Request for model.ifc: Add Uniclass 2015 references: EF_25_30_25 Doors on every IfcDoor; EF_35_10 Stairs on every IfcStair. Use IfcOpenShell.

First a look at what the model holds.

```python
import ifcopenshell

model = ifcopenshell.open("model.ifc")
print(model.schema)
print("classifications:", [c.Name for c in model.by_type("IfcClassification")])
for ifc_class in ("IfcDoor", "IfcRoof", "IfcStair", "IfcWall", "IfcWindow"):
    print(ifc_class, len(model.by_type(ifc_class)))
```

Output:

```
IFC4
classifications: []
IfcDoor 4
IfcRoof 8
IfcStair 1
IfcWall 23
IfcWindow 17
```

```python
import ifcopenshell
import ifcopenshell.api.classification

model = ifcopenshell.open("model.ifc")

system = ifcopenshell.api.classification.add_classification(model, classification="Uniclass 2015")

codes = {
    "IfcDoor": ("EF_25_30_25", "Doors"),
    "IfcStair": ("EF_35_10", "Stairs"),
}
for ifc_class, (code, name) in codes.items():
    products = model.by_type(ifc_class)
    ifcopenshell.api.classification.add_reference(
        model, products=products, classification=system, identification=code, name=name
    )
    print(code, len(products))

model.write("model-out.ifc")
```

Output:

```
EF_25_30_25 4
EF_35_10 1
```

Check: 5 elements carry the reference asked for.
